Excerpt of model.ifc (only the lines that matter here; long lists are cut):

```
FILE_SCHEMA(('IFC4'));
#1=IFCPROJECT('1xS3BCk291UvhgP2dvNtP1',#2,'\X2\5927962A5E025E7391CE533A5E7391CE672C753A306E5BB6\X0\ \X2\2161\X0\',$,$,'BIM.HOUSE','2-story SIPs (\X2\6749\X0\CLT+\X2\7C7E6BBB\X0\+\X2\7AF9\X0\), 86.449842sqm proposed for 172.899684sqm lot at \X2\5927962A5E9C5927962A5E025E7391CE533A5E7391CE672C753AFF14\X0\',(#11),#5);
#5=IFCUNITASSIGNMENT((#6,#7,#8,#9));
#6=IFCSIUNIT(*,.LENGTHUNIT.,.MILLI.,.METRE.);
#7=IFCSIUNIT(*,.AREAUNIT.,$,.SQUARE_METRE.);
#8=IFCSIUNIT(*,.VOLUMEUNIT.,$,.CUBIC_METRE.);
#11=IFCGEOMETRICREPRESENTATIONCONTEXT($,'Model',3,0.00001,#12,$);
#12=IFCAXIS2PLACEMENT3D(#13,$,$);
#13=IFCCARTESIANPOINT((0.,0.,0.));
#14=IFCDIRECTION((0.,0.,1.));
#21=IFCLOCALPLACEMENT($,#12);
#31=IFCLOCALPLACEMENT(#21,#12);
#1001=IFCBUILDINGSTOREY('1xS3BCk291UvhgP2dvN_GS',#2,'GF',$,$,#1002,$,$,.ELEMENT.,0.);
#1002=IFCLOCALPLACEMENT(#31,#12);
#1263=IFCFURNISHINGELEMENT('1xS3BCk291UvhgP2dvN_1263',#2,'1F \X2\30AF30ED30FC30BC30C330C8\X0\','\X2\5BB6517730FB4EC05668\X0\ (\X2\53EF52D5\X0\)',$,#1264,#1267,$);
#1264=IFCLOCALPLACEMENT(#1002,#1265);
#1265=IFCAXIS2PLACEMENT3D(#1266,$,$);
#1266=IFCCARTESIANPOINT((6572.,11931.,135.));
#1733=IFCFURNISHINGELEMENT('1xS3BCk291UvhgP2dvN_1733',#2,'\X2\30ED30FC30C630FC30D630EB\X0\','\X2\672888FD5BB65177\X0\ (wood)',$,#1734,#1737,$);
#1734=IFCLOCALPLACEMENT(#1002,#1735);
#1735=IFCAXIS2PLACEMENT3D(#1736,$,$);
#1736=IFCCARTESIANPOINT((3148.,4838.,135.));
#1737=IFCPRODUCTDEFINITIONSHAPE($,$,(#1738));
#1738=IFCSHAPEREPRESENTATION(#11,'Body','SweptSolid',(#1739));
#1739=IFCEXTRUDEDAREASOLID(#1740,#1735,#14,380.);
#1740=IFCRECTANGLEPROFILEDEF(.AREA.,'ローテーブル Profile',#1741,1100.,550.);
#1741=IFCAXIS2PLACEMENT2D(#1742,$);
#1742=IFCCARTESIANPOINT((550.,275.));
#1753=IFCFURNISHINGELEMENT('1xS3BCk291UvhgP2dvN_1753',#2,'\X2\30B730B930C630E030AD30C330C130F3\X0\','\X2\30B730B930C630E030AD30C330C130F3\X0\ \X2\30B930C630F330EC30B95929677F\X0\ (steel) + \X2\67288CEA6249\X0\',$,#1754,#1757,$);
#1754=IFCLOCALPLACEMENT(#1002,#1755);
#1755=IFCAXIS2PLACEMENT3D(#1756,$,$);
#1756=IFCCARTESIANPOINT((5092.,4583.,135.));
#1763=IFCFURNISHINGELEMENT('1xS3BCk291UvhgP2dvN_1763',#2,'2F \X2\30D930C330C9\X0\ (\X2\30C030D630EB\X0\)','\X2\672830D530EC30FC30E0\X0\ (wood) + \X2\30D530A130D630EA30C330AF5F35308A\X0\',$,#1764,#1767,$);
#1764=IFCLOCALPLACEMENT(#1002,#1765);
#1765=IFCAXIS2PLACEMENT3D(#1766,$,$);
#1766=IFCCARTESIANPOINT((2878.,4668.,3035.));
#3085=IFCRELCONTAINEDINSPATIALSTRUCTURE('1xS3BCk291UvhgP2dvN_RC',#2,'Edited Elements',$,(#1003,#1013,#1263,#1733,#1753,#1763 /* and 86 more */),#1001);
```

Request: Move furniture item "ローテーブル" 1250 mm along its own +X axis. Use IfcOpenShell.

```python
import ifcopenshell
import ifcopenshell.api.geometry
import ifcopenshell.util.placement

model = ifcopenshell.open("model.ifc")

item = model.by_id(1733)
matrix = ifcopenshell.util.placement.get_local_placement(item.ObjectPlacement)
matrix[:3, 3] += matrix[:3, 0] * 1250.0
ifcopenshell.api.geometry.edit_object_placement(model, product=item, matrix=matrix, is_si=False)

print(ifcopenshell.util.placement.get_local_placement(item.ObjectPlacement).round(3) + 0.0)

model.write("model-out.ifc")
```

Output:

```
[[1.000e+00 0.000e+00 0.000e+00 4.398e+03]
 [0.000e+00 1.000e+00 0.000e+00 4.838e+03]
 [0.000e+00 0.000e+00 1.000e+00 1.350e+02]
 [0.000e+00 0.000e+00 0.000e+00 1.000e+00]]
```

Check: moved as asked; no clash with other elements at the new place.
